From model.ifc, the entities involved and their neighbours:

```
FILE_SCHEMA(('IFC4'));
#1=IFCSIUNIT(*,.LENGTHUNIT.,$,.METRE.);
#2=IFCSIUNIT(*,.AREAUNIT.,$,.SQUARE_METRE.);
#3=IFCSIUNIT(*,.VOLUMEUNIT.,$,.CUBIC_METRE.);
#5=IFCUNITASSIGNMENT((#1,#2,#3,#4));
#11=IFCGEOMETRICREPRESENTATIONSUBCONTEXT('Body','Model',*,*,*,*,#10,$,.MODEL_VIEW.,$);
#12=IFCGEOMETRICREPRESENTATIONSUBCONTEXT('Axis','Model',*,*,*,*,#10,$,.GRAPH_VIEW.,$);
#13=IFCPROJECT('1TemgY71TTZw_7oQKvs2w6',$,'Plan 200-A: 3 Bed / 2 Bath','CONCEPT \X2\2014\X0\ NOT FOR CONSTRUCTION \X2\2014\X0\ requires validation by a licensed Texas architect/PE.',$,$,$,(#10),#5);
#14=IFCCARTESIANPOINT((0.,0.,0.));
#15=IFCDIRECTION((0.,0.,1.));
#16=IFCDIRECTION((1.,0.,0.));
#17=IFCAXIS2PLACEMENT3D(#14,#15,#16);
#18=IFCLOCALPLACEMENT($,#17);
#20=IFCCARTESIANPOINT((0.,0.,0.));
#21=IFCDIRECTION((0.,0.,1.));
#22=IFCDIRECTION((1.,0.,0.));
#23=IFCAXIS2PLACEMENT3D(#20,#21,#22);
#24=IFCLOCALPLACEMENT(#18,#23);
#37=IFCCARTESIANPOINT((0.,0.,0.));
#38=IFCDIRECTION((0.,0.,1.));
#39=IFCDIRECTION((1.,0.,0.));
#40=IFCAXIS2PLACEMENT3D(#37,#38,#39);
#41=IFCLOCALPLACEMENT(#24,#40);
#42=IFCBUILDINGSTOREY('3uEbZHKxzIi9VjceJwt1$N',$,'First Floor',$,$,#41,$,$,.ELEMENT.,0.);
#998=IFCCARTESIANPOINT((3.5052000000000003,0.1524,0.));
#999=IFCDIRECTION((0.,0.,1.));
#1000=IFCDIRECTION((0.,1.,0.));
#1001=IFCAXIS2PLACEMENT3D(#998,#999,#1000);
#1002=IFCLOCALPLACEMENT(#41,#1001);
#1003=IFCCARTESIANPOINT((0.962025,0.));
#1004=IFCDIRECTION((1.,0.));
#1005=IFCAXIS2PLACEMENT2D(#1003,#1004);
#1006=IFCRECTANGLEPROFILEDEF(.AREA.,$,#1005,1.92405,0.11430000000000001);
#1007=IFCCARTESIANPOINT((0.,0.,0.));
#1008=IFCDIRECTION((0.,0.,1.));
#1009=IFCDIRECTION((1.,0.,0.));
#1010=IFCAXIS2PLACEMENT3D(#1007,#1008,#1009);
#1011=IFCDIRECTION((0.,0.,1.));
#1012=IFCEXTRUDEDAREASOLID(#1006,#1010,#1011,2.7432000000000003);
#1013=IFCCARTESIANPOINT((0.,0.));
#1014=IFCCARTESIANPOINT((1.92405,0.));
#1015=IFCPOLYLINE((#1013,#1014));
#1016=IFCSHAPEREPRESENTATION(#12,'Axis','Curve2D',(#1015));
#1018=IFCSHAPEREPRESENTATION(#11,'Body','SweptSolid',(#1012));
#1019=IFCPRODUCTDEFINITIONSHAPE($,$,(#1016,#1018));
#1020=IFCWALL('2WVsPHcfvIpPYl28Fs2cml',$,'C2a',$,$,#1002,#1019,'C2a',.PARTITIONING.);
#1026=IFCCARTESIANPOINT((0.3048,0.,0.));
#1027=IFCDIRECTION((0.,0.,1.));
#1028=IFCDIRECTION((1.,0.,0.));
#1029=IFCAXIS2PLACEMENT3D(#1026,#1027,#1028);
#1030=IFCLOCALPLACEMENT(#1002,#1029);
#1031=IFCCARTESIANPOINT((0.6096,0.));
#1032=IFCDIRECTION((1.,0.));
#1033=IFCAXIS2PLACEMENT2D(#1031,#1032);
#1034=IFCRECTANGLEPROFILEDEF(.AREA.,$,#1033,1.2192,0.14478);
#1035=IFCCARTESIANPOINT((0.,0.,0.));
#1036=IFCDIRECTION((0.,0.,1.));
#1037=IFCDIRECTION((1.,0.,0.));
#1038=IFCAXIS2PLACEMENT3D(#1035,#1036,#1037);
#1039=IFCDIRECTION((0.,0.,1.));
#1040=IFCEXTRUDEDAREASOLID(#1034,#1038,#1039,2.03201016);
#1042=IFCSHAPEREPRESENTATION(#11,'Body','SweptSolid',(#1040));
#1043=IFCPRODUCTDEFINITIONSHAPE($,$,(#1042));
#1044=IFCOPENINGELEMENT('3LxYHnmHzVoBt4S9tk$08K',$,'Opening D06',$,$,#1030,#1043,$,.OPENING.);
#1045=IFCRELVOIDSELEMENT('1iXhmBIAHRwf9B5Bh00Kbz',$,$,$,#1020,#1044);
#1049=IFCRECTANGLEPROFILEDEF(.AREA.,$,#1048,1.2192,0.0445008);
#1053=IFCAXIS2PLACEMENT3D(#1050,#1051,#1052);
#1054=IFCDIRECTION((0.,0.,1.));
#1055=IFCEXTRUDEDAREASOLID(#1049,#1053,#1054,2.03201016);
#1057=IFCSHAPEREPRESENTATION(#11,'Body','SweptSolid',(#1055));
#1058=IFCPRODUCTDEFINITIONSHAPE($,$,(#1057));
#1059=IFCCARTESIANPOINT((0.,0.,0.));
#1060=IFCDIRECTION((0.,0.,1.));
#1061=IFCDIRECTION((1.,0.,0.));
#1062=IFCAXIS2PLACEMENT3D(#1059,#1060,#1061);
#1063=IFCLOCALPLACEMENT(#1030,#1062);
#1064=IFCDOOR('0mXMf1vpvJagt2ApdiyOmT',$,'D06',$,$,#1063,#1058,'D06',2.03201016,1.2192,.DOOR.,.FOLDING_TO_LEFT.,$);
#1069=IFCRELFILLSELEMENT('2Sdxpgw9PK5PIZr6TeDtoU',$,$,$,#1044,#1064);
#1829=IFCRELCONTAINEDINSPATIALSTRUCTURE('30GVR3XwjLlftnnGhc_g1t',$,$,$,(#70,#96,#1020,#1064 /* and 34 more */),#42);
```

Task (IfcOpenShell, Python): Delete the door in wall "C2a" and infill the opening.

```python
import ifcopenshell
import ifcopenshell.api.feature
import ifcopenshell.api.root
import ifcopenshell.geom
import ifcopenshell.util.shape

model = ifcopenshell.open("model.ifc")
settings = ifcopenshell.geom.settings()


def volume(element):
    """Net volume in cubic metres, openings subtracted."""
    shape = ifcopenshell.geom.create_shape(settings, element)
    return ifcopenshell.util.shape.get_volume(shape.geometry)


door = model.by_guid("0mXMf1vpvJagt2ApdiyOmT")
opening = door.FillsVoids[0].RelatingOpeningElement
wall = opening.VoidsElements[0].RelatingBuildingElement
before = volume(wall)

ifcopenshell.api.root.remove_product(model, product=door)
ifcopenshell.api.feature.remove_feature(model, feature=opening)

after = volume(wall)

print(f"wall volume {before:.3f} -> {after:.3f} m3")

model.write("model-out.ifc")
```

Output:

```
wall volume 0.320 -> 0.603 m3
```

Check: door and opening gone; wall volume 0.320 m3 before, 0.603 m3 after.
